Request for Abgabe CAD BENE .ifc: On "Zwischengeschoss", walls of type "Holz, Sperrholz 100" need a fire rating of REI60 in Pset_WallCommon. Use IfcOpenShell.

First a look at what the model holds.

```python
import ifcopenshell
import ifcopenshell.util.element

model = ifcopenshell.open("Abgabe CAD BENE .ifc")
print(model.schema)
storey = next(s for s in model.by_type("IfcBuildingStorey") if s.Name == "Zwischengeschoss")
walls = [e for e in ifcopenshell.util.element.get_decomposition(storey) if e.is_a("IfcWall")]
seen = {}
for e in walls:
    element_type = ifcopenshell.util.element.get_type(e)
    key = (element_type.Name if element_type != e and element_type else None, ifcopenshell.util.element.get_pset(e, "Pset_WallCommon", "FireRating"))
    seen[key] = seen.get(key, 0) + 1
for (name, value), count in sorted(seen.items(), key=str):
    print(count, "x", name, "|", value)
```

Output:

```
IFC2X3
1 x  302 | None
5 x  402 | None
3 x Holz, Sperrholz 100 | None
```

```python
import ifcopenshell
import ifcopenshell.api.pset
import ifcopenshell.util.element

model = ifcopenshell.open("Abgabe CAD BENE .ifc")

storey = next(s for s in model.by_type("IfcBuildingStorey") if s.Name == "Zwischengeschoss")
walls = [e for e in ifcopenshell.util.element.get_decomposition(storey) if e.is_a("IfcWall")]

count = 0
for e in walls:
    element_type = ifcopenshell.util.element.get_type(e)
    if element_type in (None, e) or element_type.Name != "Holz, Sperrholz 100":
        continue
    # add_pset returns the element's existing set when there is one.
    pset = ifcopenshell.api.pset.add_pset(model, product=e, name="Pset_WallCommon")
    ifcopenshell.api.pset.edit_pset(model, pset=pset, properties={"FireRating": "REI60"})
    count += 1

print(count, "walls updated")

model.write("Abgabe CAD BENE _edited.ifc")
```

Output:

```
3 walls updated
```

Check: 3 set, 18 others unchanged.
